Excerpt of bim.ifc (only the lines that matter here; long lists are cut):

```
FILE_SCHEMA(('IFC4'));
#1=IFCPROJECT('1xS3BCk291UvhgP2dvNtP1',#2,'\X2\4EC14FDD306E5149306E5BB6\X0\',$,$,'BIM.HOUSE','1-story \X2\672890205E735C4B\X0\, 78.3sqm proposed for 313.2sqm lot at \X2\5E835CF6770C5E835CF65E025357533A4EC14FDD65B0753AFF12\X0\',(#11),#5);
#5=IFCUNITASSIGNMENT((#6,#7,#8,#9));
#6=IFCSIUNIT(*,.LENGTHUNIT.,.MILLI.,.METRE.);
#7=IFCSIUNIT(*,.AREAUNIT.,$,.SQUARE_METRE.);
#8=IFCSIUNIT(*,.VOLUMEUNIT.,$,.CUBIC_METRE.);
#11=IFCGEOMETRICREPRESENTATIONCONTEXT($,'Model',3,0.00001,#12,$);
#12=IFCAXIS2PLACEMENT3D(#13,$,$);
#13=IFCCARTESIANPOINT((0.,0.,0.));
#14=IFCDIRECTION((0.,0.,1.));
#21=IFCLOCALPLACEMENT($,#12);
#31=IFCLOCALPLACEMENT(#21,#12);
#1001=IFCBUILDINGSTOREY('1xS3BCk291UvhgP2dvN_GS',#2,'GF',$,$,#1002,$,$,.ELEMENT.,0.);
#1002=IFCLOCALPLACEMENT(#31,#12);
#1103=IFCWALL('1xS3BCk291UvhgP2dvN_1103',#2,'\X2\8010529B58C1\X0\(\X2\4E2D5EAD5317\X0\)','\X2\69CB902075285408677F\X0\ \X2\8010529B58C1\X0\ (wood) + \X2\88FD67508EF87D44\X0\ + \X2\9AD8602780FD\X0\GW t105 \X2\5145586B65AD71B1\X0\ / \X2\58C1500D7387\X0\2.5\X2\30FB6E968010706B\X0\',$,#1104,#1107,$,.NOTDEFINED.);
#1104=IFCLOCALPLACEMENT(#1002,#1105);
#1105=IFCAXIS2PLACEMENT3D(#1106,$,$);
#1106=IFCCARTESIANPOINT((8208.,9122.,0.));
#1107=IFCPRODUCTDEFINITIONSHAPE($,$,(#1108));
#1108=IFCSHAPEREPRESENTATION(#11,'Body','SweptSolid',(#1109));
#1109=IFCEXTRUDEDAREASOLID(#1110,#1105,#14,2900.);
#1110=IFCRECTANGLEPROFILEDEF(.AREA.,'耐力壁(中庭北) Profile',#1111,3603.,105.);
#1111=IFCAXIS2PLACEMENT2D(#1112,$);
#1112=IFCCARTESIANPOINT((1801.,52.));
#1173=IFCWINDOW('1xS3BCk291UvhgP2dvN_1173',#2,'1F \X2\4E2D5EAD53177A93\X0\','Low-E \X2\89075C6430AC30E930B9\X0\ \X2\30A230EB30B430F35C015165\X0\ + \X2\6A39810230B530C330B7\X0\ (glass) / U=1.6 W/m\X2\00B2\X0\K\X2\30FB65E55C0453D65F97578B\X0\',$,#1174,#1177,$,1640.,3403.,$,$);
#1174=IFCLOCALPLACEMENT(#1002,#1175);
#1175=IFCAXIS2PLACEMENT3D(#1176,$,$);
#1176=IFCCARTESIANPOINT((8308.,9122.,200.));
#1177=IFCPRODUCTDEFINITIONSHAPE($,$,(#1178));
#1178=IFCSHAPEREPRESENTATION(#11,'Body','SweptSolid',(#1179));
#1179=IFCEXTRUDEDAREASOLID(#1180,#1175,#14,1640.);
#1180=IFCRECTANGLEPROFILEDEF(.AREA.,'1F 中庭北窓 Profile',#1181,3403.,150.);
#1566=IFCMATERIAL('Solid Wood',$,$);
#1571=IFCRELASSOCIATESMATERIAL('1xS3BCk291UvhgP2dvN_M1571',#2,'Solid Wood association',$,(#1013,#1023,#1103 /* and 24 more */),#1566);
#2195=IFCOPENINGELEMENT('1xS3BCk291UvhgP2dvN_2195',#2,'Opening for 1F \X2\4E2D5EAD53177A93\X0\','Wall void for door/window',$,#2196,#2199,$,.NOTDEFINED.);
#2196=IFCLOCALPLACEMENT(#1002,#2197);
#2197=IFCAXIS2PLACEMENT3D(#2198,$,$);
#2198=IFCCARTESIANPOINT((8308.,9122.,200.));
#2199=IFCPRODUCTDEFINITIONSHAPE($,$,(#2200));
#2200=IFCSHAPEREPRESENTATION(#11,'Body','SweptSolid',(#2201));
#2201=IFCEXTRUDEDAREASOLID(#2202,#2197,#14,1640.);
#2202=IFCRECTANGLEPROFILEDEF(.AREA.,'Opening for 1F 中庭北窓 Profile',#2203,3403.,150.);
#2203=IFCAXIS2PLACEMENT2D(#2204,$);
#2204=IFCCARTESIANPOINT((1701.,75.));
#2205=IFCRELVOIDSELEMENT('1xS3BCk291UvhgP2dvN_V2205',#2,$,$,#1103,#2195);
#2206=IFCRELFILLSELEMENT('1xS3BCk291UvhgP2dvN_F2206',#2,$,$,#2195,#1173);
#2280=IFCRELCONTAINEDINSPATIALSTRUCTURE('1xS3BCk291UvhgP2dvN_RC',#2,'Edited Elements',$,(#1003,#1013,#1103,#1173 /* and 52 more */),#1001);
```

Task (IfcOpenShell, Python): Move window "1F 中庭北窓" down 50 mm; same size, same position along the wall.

```python
import numpy as np
import ifcopenshell
import ifcopenshell.api.geometry
import ifcopenshell.util.placement
import ifcopenshell.util.unit

model = ifcopenshell.open("bim.ifc")
unit_scale = ifcopenshell.util.unit.calculate_unit_scale(model)

window = model.by_guid("1xS3BCk291UvhgP2dvN_1173")
opening = window.FillsVoids[0].RelatingOpeningElement
dz = -50.0

shift = np.array([0.0, 0.0, dz])
# The window is not placed relative to its opening, so move both.
for product in (opening, window):
    matrix = ifcopenshell.util.placement.get_local_placement(product.ObjectPlacement)
    matrix[:3, 3] += shift
    ifcopenshell.api.geometry.edit_object_placement(model, product=product, matrix=matrix, is_si=False)

print(f"moved by {dz * unit_scale:+.3f} m")

model.write("bim_updated.ifc")
```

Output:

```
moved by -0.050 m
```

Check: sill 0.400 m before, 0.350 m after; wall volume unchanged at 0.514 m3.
